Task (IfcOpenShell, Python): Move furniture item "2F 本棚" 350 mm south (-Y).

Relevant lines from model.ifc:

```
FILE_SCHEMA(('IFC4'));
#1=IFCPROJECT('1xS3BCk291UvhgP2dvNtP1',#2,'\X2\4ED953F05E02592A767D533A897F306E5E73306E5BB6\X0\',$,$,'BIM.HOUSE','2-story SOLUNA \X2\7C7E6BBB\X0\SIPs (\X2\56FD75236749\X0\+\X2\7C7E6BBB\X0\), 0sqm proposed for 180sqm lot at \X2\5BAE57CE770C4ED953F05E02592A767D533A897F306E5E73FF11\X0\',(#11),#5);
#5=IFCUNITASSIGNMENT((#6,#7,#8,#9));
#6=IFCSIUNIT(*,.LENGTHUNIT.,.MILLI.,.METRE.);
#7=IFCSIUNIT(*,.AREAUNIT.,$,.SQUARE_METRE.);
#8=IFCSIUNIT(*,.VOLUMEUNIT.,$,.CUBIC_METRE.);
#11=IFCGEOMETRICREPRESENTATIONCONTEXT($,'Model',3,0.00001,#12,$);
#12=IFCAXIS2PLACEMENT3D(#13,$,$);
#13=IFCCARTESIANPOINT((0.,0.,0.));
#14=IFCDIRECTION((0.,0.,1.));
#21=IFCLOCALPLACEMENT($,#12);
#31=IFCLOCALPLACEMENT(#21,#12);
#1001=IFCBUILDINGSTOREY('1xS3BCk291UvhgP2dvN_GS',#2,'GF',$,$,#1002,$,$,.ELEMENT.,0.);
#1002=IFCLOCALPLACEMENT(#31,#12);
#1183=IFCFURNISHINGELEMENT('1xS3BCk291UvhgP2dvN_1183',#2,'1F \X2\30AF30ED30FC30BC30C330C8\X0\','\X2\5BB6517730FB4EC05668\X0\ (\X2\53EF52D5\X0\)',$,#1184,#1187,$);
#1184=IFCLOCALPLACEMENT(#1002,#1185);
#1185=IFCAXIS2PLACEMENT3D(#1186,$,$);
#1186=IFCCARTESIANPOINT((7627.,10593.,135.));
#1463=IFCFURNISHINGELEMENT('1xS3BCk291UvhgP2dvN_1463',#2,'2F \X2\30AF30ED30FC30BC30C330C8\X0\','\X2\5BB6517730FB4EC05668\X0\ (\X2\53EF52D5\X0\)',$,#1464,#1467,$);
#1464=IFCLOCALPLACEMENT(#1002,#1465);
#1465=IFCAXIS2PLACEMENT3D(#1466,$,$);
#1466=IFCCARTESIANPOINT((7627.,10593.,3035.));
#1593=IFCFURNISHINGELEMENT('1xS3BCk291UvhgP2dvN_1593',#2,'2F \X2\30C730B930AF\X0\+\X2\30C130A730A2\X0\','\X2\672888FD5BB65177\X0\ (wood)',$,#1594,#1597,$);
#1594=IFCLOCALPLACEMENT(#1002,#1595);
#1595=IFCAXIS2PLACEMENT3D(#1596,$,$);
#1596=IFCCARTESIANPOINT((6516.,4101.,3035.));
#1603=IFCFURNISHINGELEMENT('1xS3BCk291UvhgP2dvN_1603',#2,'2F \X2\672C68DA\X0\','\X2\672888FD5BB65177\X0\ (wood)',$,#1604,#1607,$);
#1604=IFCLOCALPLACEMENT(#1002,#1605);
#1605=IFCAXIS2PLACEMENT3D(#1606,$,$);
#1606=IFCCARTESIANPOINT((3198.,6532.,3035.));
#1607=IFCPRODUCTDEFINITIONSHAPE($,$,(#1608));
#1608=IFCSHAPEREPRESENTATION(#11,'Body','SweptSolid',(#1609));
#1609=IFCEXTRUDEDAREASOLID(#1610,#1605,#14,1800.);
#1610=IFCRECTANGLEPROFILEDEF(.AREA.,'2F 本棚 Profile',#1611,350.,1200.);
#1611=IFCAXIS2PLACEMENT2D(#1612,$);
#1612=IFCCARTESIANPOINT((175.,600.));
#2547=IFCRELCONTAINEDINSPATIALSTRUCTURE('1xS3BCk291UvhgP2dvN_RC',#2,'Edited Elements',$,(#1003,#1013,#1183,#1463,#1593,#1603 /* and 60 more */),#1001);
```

```python
import ifcopenshell
import ifcopenshell.api.geometry
import ifcopenshell.util.placement
import ifcopenshell.util.unit

model = ifcopenshell.open("model.ifc")
unit_scale = ifcopenshell.util.unit.calculate_unit_scale(model)

item = model.by_id(1603)
matrix = ifcopenshell.util.placement.get_local_placement(item.ObjectPlacement)
matrix[1, 3] -= 0.35 / unit_scale
ifcopenshell.api.geometry.edit_object_placement(model, product=item, matrix=matrix, is_si=False)

print(ifcopenshell.util.placement.get_local_placement(item.ObjectPlacement).round(3) + 0.0)

model.write("model-out.ifc")
```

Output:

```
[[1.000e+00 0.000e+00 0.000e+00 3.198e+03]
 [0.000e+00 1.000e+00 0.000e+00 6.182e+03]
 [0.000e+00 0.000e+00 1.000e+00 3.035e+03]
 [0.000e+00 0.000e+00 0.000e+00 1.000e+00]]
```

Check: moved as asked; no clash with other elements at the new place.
